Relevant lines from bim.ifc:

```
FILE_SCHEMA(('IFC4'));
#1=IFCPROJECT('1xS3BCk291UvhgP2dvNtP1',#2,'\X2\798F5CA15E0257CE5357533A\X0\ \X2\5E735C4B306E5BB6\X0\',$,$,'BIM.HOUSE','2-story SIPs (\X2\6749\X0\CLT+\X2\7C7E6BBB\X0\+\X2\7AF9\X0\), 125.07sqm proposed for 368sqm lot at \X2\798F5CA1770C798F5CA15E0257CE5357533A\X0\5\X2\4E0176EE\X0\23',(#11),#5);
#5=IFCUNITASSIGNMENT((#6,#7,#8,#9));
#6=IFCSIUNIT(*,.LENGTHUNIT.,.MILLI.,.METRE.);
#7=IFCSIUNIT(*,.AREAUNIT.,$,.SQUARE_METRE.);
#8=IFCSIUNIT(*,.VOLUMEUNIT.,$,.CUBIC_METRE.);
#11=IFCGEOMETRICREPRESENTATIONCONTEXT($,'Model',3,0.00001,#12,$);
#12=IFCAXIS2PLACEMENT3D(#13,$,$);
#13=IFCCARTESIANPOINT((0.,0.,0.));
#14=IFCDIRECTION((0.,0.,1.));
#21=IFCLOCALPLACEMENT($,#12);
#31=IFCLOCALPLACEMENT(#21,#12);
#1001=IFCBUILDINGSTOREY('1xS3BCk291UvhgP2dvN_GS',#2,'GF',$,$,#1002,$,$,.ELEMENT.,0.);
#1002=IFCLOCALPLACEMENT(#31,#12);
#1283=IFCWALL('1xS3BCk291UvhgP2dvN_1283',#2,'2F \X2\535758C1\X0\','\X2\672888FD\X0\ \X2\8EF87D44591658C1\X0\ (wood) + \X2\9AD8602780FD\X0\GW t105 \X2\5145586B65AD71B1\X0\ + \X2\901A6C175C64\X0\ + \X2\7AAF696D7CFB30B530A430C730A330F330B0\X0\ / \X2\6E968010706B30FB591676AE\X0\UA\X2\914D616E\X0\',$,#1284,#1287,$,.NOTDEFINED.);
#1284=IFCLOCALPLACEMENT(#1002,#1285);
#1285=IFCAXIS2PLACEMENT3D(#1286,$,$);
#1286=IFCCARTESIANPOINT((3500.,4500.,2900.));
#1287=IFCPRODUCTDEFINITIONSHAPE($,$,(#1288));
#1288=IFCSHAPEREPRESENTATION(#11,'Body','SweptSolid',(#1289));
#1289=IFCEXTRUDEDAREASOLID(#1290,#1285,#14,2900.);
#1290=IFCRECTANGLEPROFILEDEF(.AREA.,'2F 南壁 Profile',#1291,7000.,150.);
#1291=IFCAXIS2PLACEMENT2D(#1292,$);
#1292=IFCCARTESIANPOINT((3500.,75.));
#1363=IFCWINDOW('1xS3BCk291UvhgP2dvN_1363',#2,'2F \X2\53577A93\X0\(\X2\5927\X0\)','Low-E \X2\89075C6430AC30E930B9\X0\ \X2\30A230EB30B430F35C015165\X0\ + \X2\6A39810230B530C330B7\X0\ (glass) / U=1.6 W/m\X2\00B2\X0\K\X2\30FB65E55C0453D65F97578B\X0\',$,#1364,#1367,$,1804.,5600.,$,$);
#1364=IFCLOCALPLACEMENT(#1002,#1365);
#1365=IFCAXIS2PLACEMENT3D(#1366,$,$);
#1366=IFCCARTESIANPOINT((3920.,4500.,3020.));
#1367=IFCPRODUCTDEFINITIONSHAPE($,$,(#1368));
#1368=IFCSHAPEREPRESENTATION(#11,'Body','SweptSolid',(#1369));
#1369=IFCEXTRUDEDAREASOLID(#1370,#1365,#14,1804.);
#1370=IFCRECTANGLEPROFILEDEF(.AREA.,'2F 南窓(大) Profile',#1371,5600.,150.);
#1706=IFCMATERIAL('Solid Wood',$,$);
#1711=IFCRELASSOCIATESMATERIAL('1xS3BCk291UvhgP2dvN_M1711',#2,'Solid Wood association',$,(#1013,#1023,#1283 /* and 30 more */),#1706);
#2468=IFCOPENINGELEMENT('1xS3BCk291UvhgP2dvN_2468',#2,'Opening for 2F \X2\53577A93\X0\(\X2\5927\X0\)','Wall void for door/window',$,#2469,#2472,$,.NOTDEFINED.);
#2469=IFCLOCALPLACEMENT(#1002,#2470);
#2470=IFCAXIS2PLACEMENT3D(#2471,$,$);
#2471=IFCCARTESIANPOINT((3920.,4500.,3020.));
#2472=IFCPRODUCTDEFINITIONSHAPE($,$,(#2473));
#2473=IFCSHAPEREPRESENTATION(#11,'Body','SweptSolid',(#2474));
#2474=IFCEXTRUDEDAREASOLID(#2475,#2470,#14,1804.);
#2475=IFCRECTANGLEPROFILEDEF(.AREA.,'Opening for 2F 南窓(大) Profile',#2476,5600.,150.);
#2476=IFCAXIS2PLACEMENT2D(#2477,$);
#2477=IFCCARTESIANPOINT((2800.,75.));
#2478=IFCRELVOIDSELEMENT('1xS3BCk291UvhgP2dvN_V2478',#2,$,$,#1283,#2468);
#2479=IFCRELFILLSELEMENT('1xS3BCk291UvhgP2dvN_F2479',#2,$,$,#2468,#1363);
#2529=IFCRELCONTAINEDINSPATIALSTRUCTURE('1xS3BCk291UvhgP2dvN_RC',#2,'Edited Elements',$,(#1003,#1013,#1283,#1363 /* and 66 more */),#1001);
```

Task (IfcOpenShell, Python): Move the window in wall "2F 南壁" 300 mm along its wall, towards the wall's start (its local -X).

```python
import ifcopenshell
import ifcopenshell.api.geometry
import ifcopenshell.util.placement
import ifcopenshell.util.unit

model = ifcopenshell.open("bim.ifc")
unit_scale = ifcopenshell.util.unit.calculate_unit_scale(model)

window = model.by_id(1363)
opening = window.FillsVoids[0].RelatingOpeningElement
wall = opening.VoidsElements[0].RelatingBuildingElement

wall_matrix = ifcopenshell.util.placement.get_local_placement(wall.ObjectPlacement)
shift = wall_matrix[:3, 0] * -0.3 / unit_scale
before = ifcopenshell.util.placement.get_local_placement(window.ObjectPlacement)[:3, 3].copy()

# The window is not placed relative to its opening, so move both.
for product in (opening, window):
    matrix = ifcopenshell.util.placement.get_local_placement(product.ObjectPlacement)
    matrix[:3, 3] += shift
    ifcopenshell.api.geometry.edit_object_placement(model, product=product, matrix=matrix, is_si=False)

after = ifcopenshell.util.placement.get_local_placement(window.ObjectPlacement)[:3, 3]
print("window moved by", (after - before).round(3) + 0.0)

model.write("bim_v2.ifc")
```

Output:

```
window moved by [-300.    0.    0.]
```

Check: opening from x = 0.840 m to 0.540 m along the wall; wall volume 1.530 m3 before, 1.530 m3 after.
